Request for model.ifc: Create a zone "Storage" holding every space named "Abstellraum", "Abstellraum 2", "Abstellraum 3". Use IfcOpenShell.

First a look at what the model holds.

```python
import ifcopenshell

model = ifcopenshell.open("model.ifc")
print(model.schema)
seen = {}
for space in model.by_type("IfcSpace"):
    seen[space.Name] = seen.get(space.Name, 0) + 1
for name, count in sorted(seen.items(), key=str):
    print(count, "x", name)
print("zones:", [z.Name for z in model.by_type("IfcZone")][:20])
```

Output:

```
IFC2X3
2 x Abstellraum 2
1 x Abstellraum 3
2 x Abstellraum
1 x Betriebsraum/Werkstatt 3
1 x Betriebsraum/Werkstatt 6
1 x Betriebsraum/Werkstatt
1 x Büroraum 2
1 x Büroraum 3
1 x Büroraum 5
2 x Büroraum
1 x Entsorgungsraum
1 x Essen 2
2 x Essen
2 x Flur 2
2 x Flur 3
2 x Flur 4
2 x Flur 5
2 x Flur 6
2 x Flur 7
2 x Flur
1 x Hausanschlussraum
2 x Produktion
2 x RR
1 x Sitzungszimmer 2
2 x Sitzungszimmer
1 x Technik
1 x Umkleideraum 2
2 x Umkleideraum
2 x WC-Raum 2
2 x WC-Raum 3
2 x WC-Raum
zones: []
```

```python
import ifcopenshell
import ifcopenshell.api.group
import ifcopenshell.api.root

model = ifcopenshell.open("model.ifc")

names = {"Abstellraum", "Abstellraum 2", "Abstellraum 3"}
spaces = [s for s in model.by_type("IfcSpace") if s.Name in names]

zone = ifcopenshell.api.root.create_entity(model, ifc_class="IfcZone", name="Storage")
ifcopenshell.api.group.assign_group(model, products=spaces, group=zone)
print(len(spaces), "spaces in", zone.Name)

model.write("model_rev.ifc")
```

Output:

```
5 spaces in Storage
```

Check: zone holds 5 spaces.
